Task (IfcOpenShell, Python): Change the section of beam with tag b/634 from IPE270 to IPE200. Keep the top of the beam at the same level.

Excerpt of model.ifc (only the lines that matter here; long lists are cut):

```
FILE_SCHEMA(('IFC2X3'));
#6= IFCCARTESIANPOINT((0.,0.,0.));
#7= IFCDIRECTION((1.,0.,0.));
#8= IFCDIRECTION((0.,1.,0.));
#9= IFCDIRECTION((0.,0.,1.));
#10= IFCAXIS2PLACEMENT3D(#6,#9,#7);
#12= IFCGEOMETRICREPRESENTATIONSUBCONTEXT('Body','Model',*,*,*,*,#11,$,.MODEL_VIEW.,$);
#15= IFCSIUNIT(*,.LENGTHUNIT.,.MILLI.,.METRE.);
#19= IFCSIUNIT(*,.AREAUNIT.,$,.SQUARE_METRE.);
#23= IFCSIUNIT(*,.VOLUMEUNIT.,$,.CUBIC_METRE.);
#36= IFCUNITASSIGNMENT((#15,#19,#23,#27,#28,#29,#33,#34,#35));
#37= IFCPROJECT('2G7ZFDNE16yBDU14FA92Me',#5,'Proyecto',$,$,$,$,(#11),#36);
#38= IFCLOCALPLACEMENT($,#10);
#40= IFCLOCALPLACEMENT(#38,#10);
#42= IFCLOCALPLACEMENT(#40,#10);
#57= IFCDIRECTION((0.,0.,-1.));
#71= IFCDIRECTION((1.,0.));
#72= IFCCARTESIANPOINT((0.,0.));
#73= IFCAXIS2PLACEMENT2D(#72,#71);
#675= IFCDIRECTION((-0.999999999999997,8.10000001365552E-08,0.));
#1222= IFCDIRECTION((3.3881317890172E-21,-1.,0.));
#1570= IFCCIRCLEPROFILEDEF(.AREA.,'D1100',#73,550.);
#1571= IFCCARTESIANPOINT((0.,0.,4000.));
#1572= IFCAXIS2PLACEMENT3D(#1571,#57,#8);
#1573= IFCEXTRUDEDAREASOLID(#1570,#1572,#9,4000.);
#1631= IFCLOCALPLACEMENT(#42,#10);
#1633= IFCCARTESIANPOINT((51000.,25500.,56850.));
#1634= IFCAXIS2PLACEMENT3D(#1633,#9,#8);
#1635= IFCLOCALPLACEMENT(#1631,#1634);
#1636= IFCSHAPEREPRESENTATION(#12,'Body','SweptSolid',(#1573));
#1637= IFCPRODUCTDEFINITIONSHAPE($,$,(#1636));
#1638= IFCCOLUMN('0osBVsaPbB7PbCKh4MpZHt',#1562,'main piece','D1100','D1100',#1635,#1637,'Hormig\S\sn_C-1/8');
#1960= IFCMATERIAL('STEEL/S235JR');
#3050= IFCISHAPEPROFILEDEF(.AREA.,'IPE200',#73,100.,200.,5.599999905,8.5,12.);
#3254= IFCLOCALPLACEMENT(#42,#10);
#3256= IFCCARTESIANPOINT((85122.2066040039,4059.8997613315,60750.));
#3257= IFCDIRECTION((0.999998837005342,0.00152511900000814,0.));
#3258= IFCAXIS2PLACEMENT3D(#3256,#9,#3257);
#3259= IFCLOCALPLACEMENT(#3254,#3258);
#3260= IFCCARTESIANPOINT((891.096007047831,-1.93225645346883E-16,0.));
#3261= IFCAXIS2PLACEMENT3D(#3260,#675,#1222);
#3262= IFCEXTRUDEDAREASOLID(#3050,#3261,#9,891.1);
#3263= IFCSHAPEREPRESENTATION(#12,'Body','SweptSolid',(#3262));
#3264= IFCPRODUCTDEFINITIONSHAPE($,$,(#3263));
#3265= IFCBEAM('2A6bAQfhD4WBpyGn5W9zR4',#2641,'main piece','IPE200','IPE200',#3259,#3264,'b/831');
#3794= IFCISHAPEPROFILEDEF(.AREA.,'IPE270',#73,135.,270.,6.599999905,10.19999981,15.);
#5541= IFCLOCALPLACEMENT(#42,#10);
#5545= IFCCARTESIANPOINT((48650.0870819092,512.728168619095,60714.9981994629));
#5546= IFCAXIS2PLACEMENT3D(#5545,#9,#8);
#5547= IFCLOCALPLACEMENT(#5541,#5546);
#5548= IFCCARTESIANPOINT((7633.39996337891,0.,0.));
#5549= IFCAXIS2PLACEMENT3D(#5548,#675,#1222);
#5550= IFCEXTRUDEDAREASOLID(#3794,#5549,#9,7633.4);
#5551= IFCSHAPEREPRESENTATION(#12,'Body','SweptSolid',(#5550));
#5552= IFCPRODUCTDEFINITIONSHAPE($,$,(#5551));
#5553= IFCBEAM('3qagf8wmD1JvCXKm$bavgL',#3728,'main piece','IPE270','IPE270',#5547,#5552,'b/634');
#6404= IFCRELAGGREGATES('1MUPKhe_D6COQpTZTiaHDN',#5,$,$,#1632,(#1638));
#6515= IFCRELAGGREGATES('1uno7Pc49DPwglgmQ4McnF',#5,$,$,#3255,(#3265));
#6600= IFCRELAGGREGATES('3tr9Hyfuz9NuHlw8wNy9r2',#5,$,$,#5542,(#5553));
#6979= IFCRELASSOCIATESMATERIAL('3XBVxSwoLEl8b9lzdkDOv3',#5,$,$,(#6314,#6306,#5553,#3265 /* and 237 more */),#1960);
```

```python
import ifcopenshell
import ifcopenshell.util.element
import ifcopenshell.util.representation

model = ifcopenshell.open("model.ifc")

member = model.by_guid("3qagf8wmD1JvCXKm$bavgL")
source = next(p for p in model.by_type("IfcIShapeProfileDef") if p.ProfileName == "IPE200")

body = ifcopenshell.util.representation.get_representation(member, "Model", "Body")
solid = body.Items[0]
old_profile = solid.SweptArea

# Copy the section's sizes but keep this member's own profile position.
profile = ifcopenshell.util.element.copy(model, source)
# Profiles are centred, so shift by half the change in depth to hold the top.
shift = (old_profile.OverallDepth - profile.OverallDepth) / 2
x, y = old_profile.Position.Location.Coordinates
up = (0.0, 1.0)  # upwards, in the solid's own plane
location = model.createIfcCartesianPoint((x + up[0] * shift, y + up[1] * shift))
profile.Position = model.createIfcAxis2Placement2D(location, old_profile.Position.RefDirection)
solid.SweptArea = profile
if not model.get_total_inverses(old_profile):
    ifcopenshell.util.element.remove_deep2(model, old_profile)
member.Description = member.Description.replace("IPE270", "IPE200")
member.ObjectType = member.ObjectType.replace("IPE270", "IPE200")

print(solid.SweptArea)

model.write("model_edited.ifc")
```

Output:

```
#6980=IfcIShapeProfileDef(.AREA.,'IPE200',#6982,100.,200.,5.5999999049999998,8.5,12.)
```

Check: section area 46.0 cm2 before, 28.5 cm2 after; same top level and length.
